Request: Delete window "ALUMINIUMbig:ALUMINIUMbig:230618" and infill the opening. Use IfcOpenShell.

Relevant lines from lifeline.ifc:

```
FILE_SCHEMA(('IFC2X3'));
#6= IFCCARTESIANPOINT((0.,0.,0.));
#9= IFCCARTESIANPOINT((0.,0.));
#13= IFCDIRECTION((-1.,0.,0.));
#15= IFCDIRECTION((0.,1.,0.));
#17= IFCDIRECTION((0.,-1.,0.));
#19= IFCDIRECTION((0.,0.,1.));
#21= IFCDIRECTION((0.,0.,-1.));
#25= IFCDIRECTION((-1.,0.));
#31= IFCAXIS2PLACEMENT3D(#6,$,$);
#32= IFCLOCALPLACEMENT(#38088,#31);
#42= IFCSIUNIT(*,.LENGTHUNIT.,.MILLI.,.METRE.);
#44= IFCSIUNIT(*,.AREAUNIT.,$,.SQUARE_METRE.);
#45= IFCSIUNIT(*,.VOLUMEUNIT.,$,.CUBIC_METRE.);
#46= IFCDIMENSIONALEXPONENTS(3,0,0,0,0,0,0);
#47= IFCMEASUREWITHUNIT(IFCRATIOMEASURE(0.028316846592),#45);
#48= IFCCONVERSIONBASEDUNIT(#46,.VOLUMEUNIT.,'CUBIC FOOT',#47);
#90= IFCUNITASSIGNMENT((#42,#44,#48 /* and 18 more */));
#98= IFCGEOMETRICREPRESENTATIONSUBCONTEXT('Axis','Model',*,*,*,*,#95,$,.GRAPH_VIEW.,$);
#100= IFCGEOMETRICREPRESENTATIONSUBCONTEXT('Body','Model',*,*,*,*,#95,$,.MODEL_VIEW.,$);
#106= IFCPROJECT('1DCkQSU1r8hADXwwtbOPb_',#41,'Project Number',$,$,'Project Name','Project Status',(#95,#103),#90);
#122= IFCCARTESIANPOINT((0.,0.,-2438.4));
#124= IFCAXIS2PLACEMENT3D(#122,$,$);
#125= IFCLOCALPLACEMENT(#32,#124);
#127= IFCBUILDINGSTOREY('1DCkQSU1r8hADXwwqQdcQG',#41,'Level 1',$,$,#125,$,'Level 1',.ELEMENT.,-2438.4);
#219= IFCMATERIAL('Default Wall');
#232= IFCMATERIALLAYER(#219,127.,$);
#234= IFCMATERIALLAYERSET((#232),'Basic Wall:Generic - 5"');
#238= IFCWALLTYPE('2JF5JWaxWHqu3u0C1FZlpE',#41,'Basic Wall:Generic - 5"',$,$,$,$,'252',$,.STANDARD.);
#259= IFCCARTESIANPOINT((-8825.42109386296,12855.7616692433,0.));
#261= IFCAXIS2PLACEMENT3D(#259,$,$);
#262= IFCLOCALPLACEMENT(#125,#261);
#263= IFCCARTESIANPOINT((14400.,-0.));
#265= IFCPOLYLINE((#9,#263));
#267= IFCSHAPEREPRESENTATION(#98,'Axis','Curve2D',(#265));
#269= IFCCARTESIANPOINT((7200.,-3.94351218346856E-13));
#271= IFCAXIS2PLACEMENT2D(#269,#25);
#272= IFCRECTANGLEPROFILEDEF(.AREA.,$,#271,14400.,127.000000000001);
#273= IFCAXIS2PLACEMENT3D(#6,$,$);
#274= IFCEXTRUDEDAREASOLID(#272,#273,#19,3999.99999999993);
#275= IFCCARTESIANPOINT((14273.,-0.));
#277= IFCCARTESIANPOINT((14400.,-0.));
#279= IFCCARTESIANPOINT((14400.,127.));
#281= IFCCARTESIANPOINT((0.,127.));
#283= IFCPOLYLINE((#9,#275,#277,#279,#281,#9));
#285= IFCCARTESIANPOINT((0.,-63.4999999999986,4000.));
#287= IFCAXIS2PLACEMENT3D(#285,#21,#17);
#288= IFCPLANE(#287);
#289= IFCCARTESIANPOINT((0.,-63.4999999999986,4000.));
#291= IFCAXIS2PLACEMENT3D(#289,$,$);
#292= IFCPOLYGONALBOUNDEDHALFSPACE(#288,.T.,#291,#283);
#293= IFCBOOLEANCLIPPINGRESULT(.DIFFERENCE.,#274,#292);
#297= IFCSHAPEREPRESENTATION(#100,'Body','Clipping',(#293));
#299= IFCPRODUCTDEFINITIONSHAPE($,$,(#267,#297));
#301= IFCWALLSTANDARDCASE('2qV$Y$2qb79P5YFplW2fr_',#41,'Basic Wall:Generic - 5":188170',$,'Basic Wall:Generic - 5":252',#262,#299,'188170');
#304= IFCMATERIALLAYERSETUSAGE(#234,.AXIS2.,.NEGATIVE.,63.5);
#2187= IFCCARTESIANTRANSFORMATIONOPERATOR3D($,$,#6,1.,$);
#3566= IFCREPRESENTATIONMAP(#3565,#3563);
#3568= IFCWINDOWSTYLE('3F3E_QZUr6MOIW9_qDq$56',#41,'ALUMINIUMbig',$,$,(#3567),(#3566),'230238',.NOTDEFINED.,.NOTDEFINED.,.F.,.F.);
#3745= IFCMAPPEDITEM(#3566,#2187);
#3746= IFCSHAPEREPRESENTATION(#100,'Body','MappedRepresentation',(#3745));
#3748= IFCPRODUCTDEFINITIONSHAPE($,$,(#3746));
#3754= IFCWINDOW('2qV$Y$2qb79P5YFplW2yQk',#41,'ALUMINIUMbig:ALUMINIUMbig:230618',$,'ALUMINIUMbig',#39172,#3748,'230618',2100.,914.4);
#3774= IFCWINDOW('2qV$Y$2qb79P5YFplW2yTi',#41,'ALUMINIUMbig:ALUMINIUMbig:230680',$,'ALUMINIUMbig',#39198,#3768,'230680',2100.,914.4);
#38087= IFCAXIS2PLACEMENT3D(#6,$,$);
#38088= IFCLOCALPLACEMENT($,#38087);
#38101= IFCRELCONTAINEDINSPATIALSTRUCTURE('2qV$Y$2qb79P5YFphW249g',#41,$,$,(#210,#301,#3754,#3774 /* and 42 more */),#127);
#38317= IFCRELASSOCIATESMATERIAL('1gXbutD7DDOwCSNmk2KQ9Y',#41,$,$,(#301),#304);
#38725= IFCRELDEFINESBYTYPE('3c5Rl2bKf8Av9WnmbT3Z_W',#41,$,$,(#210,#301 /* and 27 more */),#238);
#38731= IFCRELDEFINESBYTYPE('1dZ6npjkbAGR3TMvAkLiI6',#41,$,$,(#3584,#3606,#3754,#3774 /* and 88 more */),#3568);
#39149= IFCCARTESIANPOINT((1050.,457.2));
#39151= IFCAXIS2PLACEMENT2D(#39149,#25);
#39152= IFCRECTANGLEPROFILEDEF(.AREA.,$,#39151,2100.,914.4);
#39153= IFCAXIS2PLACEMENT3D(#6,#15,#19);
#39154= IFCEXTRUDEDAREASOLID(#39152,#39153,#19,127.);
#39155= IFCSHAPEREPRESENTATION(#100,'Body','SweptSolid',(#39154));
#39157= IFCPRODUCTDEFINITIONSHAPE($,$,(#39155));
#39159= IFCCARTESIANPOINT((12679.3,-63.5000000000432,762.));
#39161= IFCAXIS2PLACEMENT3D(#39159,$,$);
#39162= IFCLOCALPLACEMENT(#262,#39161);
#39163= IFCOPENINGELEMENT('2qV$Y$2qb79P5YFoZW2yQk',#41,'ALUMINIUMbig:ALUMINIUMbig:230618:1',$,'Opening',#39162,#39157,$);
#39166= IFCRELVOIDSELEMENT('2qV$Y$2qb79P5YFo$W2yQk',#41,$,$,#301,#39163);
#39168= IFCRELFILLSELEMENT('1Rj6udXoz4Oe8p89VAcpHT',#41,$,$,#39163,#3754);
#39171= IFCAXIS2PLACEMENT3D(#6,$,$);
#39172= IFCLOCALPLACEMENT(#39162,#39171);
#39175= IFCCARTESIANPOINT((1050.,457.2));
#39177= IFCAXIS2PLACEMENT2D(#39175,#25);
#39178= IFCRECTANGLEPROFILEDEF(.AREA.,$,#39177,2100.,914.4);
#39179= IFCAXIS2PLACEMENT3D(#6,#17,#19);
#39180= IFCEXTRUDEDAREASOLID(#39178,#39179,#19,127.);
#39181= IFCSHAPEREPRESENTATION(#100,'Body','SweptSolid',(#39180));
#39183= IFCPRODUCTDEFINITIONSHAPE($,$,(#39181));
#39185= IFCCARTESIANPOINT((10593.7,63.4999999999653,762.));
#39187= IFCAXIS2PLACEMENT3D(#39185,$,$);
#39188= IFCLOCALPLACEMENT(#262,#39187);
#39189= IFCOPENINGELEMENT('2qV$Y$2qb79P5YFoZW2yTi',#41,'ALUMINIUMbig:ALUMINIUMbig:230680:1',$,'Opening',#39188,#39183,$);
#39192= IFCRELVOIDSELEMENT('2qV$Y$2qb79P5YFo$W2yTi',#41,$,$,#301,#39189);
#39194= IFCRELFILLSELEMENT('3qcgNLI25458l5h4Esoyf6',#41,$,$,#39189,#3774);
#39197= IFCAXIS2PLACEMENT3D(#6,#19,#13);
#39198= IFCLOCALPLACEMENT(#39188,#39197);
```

```python
import ifcopenshell
import ifcopenshell.api.feature
import ifcopenshell.api.root
import ifcopenshell.geom
import ifcopenshell.util.shape

model = ifcopenshell.open("lifeline.ifc")
settings = ifcopenshell.geom.settings()


def volume(element):
    """Net volume in cubic metres, openings subtracted."""
    shape = ifcopenshell.geom.create_shape(settings, element)
    return ifcopenshell.util.shape.get_volume(shape.geometry)


window = model.by_guid("2qV$Y$2qb79P5YFplW2yQk")
opening = window.FillsVoids[0].RelatingOpeningElement
wall = opening.VoidsElements[0].RelatingBuildingElement
before = volume(wall)

ifcopenshell.api.root.remove_product(model, product=window)
ifcopenshell.api.feature.remove_feature(model, feature=opening)

after = volume(wall)

print(f"wall volume {before:.3f} -> {after:.3f} m3")

model.write("lifeline_updated.ifc")
```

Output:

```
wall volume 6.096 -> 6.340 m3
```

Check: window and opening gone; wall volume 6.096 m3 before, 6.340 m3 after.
